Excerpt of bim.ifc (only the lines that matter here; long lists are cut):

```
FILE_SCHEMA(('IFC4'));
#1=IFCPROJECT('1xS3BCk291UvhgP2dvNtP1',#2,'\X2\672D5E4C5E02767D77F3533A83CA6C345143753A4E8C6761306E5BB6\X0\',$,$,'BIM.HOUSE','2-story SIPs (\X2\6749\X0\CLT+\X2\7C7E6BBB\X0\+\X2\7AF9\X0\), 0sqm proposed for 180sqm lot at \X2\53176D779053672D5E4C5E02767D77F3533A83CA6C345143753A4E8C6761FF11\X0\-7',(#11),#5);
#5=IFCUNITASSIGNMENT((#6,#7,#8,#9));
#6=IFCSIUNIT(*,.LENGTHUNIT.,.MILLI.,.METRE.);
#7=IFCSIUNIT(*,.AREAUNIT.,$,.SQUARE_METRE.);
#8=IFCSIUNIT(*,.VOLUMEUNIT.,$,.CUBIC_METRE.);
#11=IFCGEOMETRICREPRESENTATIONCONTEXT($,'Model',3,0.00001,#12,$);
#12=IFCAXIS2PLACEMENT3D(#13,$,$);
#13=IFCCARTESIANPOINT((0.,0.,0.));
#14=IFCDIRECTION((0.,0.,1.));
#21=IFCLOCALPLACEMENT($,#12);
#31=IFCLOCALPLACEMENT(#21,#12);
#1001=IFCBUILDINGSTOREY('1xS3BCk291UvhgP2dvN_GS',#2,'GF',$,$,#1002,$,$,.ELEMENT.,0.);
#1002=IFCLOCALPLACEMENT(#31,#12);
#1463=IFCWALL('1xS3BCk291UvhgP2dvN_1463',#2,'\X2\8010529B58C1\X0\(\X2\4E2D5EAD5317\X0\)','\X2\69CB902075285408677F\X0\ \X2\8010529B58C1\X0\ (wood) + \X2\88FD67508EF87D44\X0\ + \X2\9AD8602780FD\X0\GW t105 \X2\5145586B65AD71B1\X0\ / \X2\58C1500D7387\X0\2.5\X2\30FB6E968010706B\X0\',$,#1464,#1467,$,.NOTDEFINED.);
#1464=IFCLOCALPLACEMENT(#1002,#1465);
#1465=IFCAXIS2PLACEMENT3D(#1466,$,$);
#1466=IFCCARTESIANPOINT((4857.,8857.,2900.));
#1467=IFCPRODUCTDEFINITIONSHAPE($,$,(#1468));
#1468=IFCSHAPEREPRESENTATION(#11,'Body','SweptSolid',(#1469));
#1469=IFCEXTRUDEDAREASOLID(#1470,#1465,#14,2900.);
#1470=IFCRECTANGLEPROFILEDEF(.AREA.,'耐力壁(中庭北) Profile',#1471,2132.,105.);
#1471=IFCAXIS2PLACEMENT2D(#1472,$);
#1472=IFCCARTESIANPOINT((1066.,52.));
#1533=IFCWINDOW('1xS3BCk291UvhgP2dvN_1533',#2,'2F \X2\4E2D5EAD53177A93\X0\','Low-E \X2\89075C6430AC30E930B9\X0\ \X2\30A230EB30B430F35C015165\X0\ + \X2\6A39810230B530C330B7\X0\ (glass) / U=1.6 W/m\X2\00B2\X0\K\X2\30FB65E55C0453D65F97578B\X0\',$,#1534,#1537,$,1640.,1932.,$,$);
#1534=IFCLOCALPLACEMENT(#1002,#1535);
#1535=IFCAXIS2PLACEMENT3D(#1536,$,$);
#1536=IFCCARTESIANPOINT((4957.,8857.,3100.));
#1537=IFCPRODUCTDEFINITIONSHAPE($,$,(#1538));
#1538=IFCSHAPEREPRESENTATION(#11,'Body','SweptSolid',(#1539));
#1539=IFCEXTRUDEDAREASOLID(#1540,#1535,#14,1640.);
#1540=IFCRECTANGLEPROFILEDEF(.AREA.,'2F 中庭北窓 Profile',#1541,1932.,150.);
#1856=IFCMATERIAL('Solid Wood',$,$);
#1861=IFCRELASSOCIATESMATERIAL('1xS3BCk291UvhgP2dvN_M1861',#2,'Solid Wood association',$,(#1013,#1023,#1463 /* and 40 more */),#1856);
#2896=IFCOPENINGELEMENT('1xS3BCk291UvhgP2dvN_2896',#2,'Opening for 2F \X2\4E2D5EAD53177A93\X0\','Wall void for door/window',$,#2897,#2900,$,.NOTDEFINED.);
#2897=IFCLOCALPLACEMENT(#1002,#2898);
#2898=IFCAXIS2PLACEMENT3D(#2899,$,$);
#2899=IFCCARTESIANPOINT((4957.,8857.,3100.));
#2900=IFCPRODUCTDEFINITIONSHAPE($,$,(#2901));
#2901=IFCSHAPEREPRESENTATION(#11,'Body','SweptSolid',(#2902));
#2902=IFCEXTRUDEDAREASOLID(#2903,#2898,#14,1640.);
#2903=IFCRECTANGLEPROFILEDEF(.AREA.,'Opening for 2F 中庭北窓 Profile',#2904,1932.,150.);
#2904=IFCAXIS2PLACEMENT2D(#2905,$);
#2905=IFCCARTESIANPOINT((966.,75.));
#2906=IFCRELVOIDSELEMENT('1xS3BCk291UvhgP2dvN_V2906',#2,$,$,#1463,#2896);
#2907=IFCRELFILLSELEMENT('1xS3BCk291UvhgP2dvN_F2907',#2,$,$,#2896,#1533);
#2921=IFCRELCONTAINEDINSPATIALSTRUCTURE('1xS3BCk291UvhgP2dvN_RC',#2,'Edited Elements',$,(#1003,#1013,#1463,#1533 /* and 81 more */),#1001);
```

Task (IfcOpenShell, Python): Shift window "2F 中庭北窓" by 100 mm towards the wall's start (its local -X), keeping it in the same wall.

```python
import ifcopenshell
import ifcopenshell.api.geometry
import ifcopenshell.util.placement
import ifcopenshell.util.unit

model = ifcopenshell.open("bim.ifc")
unit_scale = ifcopenshell.util.unit.calculate_unit_scale(model)

window = model.by_guid("1xS3BCk291UvhgP2dvN_1533")
opening = window.FillsVoids[0].RelatingOpeningElement
wall = opening.VoidsElements[0].RelatingBuildingElement

wall_matrix = ifcopenshell.util.placement.get_local_placement(wall.ObjectPlacement)
shift = wall_matrix[:3, 0] * -0.1 / unit_scale
before = ifcopenshell.util.placement.get_local_placement(window.ObjectPlacement)[:3, 3].copy()

# The window is not placed relative to its opening, so move both.
for product in (opening, window):
    matrix = ifcopenshell.util.placement.get_local_placement(product.ObjectPlacement)
    matrix[:3, 3] += shift
    ifcopenshell.api.geometry.edit_object_placement(model, product=product, matrix=matrix, is_si=False)

after = ifcopenshell.util.placement.get_local_placement(window.ObjectPlacement)[:3, 3]
print("window moved by", (after - before).round(3) + 0.0)

model.write("bim_v2.ifc")
```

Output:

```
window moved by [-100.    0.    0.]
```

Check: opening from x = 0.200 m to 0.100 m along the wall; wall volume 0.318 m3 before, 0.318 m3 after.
